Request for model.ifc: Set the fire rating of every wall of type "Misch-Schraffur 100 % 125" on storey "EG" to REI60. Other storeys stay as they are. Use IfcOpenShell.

First a look at what the model holds.

```python
import ifcopenshell
import ifcopenshell.util.element

model = ifcopenshell.open("model.ifc")
print(model.schema)
storey = next(s for s in model.by_type("IfcBuildingStorey") if s.Name == "EG")
walls = [e for e in ifcopenshell.util.element.get_decomposition(storey) if e.is_a("IfcWall")]
seen = {}
for e in walls:
    element_type = ifcopenshell.util.element.get_type(e)
    key = (element_type.Name if element_type != e and element_type else None, ifcopenshell.util.element.get_pset(e, "Pset_WallCommon", "FireRating"))
    seen[key] = seen.get(key, 0) + 1
for (name, value), count in sorted(seen.items(), key=str):
    print(count, "x", name, "|", value)
```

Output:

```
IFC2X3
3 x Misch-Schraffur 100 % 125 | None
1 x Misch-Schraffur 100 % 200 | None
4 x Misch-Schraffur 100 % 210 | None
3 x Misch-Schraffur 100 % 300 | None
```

```python
import ifcopenshell
import ifcopenshell.api.pset
import ifcopenshell.util.element

model = ifcopenshell.open("model.ifc")

storey = next(s for s in model.by_type("IfcBuildingStorey") if s.Name == "EG")
walls = [e for e in ifcopenshell.util.element.get_decomposition(storey) if e.is_a("IfcWall")]

count = 0
for e in walls:
    element_type = ifcopenshell.util.element.get_type(e)
    if element_type in (None, e) or element_type.Name != "Misch-Schraffur 100 % 125":
        continue
    # add_pset returns the element's existing set when there is one.
    pset = ifcopenshell.api.pset.add_pset(model, product=e, name="Pset_WallCommon")
    ifcopenshell.api.pset.edit_pset(model, pset=pset, properties={"FireRating": "REI60"})
    count += 1

print(count, "walls updated")

model.write("model_rev.ifc")
```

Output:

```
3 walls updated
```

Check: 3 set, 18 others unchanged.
